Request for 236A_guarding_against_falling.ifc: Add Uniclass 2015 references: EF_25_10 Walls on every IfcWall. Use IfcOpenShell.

First a look at what the model holds.

```python
import ifcopenshell

model = ifcopenshell.open("236A_guarding_against_falling.ifc")
print(model.schema)
print("classifications:", [c.Name for c in model.by_type("IfcClassification")])
for ifc_class in ("IfcDoor", "IfcRoof", "IfcStair", "IfcWall", "IfcWindow"):
    print(ifc_class, len(model.by_type(ifc_class)))
```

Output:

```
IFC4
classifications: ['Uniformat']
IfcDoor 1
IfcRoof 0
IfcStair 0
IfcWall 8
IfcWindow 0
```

```python
import ifcopenshell
import ifcopenshell.api.classification

model = ifcopenshell.open("236A_guarding_against_falling.ifc")

system = ifcopenshell.api.classification.add_classification(model, classification="Uniclass 2015")

codes = {
    "IfcWall": ("EF_25_10", "Walls"),
}
for ifc_class, (code, name) in codes.items():
    products = model.by_type(ifc_class)
    ifcopenshell.api.classification.add_reference(
        model, products=products, classification=system, identification=code, name=name
    )
    print(code, len(products))

model.write("236A_guarding_against_falling_v2.ifc")
```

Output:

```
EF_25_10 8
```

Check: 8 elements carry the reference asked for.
